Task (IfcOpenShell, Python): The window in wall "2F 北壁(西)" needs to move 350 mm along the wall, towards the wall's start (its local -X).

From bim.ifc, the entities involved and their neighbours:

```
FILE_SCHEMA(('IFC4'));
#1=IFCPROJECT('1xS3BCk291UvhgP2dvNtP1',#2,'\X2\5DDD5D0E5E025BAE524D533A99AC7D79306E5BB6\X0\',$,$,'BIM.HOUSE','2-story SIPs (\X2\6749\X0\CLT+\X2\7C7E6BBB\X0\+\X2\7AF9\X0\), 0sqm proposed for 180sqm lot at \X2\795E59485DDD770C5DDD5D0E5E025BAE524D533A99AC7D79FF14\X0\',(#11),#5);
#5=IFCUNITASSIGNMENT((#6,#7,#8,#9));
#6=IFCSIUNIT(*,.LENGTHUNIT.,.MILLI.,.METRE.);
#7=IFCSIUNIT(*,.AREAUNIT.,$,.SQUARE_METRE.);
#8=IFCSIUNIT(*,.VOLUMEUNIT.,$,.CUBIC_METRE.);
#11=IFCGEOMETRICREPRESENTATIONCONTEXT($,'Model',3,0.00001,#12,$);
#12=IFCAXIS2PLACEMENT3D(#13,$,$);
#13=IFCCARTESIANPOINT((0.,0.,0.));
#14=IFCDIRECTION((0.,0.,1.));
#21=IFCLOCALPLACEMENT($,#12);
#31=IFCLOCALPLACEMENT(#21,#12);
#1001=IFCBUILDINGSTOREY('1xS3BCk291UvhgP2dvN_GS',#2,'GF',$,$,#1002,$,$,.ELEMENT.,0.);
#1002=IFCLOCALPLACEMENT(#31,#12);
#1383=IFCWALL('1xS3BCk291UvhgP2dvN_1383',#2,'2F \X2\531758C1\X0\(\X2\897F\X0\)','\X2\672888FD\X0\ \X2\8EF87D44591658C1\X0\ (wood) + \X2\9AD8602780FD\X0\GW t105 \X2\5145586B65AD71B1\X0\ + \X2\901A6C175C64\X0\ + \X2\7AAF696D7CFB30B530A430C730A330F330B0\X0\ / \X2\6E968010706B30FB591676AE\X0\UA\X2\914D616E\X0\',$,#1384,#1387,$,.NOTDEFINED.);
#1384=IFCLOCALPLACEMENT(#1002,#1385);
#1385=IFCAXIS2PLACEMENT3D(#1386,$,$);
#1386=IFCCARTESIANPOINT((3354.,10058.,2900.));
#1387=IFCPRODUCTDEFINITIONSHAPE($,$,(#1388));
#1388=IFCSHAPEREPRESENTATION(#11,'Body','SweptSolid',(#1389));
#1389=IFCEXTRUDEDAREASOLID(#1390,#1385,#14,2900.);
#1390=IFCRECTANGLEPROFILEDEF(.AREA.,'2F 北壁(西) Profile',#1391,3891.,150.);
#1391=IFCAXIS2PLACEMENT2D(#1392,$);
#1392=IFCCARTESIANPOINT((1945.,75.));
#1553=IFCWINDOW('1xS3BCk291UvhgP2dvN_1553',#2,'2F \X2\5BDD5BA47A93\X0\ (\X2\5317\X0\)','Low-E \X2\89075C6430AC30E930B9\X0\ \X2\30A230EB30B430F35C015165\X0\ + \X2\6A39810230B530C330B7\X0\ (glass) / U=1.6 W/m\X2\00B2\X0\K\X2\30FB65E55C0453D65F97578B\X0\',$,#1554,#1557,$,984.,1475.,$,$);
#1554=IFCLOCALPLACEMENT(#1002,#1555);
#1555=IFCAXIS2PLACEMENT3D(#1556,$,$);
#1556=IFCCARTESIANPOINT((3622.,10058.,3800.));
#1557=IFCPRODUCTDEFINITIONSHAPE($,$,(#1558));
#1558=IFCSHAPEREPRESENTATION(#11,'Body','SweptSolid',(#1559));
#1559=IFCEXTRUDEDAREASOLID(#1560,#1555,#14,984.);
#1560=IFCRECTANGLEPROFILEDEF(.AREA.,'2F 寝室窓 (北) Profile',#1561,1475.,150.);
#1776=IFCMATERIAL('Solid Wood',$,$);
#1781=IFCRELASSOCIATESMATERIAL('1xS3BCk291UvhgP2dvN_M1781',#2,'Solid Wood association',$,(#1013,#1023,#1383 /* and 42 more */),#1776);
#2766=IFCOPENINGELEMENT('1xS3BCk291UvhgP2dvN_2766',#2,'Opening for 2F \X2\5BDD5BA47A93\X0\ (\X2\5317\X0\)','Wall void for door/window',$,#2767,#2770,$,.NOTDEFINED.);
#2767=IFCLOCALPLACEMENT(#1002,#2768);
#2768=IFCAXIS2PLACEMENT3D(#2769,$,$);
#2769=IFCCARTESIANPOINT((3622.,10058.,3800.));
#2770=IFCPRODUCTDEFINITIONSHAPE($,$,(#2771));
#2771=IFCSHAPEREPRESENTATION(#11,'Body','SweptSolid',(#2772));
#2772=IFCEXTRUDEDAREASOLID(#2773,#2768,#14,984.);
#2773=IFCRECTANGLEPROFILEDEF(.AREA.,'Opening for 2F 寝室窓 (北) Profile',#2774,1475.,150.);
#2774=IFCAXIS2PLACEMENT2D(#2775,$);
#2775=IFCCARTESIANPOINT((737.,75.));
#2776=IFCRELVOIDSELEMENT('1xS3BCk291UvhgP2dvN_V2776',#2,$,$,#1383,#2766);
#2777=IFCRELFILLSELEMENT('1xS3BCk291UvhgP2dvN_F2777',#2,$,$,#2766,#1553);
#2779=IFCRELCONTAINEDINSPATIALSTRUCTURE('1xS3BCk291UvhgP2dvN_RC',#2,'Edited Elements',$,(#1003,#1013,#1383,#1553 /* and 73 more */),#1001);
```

```python
import ifcopenshell
import ifcopenshell.api.geometry
import ifcopenshell.util.placement

model = ifcopenshell.open("bim.ifc")

window = model.by_guid("1xS3BCk291UvhgP2dvN_1553")
opening = window.FillsVoids[0].RelatingOpeningElement
wall = opening.VoidsElements[0].RelatingBuildingElement

wall_matrix = ifcopenshell.util.placement.get_local_placement(wall.ObjectPlacement)
shift = wall_matrix[:3, 0] * -350.0
before = ifcopenshell.util.placement.get_local_placement(window.ObjectPlacement)[:3, 3].copy()

# The window is not placed relative to its opening, so move both.
for product in (opening, window):
    matrix = ifcopenshell.util.placement.get_local_placement(product.ObjectPlacement)
    matrix[:3, 3] += shift
    ifcopenshell.api.geometry.edit_object_placement(model, product=product, matrix=matrix, is_si=False)

after = ifcopenshell.util.placement.get_local_placement(window.ObjectPlacement)[:3, 3]
print("window moved by", (after - before).round(3) + 0.0)

model.write("bim_v2.ifc")
```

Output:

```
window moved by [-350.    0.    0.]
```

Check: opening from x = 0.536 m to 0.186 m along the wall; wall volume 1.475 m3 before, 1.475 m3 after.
